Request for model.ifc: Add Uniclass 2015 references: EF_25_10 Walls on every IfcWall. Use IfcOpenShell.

First a look at what the model holds.

```python
import ifcopenshell

model = ifcopenshell.open("model.ifc")
print(model.schema)
print("classifications:", [c.Name for c in model.by_type("IfcClassification")])
for ifc_class in ("IfcDoor", "IfcRoof", "IfcStair", "IfcWall", "IfcWindow"):
    print(ifc_class, len(model.by_type(ifc_class)))
```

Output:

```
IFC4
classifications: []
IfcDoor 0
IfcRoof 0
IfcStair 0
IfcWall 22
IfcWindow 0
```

```python
import ifcopenshell
import ifcopenshell.api.classification

model = ifcopenshell.open("model.ifc")

system = ifcopenshell.api.classification.add_classification(model, classification="Uniclass 2015")

codes = {
    "IfcWall": ("EF_25_10", "Walls"),
}
for ifc_class, (code, name) in codes.items():
    products = model.by_type(ifc_class)
    ifcopenshell.api.classification.add_reference(
        model, products=products, classification=system, identification=code, name=name
    )
    print(code, len(products))

model.write("model_rev.ifc")
```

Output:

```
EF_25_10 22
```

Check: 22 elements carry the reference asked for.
